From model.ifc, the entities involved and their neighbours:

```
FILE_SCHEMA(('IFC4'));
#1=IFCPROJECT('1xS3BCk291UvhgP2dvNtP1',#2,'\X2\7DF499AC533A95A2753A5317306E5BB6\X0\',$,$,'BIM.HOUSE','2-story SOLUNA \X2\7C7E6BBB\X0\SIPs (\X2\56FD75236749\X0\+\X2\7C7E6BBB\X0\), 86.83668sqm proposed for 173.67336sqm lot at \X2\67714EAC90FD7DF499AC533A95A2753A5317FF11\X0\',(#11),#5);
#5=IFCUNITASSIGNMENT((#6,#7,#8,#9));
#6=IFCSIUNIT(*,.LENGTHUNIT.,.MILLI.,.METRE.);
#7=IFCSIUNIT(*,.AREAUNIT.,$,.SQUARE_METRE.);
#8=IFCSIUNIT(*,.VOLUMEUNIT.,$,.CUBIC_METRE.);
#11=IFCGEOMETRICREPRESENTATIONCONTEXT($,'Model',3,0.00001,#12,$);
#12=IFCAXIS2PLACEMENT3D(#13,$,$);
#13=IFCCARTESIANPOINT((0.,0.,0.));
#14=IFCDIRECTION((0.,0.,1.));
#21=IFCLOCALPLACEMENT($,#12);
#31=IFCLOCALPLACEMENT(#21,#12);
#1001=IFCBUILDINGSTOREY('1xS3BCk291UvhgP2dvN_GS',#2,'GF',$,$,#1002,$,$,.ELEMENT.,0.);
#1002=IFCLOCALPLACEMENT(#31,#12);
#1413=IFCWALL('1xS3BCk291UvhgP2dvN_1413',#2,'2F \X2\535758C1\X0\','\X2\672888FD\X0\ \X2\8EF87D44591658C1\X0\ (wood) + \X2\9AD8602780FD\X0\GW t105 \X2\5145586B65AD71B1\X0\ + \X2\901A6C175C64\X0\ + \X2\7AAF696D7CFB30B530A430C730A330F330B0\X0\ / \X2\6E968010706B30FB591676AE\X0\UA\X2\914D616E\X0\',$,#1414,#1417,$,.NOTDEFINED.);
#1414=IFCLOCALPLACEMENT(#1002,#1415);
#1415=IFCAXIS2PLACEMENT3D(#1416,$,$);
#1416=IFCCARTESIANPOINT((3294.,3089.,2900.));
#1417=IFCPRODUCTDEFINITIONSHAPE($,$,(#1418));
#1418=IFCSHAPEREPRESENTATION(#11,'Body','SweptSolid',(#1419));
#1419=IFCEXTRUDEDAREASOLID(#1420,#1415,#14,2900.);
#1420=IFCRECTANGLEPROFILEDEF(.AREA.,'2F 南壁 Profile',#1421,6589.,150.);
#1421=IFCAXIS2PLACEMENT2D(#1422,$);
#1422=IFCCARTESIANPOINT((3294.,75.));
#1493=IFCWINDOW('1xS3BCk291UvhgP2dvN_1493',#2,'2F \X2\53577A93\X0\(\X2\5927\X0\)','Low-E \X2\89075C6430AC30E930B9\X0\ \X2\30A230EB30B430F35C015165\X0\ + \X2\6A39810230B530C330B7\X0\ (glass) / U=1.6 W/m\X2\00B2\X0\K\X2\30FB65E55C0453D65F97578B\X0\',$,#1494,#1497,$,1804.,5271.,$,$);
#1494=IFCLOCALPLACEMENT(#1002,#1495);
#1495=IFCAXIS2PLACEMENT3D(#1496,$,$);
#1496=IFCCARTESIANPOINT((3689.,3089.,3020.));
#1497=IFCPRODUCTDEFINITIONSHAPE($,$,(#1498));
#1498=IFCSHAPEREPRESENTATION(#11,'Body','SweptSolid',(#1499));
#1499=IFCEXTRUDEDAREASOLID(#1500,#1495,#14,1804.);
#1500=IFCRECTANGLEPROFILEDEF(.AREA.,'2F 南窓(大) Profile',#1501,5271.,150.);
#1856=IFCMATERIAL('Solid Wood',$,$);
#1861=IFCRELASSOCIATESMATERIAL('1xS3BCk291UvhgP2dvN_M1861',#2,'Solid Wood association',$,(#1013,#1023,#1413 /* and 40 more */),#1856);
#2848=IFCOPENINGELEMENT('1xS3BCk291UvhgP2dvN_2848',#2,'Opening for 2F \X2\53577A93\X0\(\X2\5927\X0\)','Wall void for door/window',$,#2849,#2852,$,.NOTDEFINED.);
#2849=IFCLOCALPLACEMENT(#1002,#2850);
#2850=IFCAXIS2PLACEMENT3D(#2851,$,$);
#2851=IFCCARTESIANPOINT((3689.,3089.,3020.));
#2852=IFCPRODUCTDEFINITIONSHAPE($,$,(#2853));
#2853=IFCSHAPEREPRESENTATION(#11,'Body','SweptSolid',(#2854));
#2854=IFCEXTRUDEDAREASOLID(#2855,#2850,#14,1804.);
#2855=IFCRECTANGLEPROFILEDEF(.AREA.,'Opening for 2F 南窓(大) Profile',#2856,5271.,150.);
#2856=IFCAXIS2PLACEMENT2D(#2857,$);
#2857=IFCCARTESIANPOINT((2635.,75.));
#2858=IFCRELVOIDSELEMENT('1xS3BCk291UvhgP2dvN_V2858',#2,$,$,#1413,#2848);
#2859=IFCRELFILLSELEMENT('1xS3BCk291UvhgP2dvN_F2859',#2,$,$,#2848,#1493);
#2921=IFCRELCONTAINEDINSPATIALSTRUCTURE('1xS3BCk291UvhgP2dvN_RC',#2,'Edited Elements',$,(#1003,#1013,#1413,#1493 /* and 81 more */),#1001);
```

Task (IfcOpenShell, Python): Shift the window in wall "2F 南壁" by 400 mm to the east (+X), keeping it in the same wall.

```python
import ifcopenshell
import ifcopenshell.api.geometry
import ifcopenshell.util.placement

model = ifcopenshell.open("model.ifc")

window = model.by_guid("1xS3BCk291UvhgP2dvN_1493")
opening = window.FillsVoids[0].RelatingOpeningElement
wall = opening.VoidsElements[0].RelatingBuildingElement

wall_matrix = ifcopenshell.util.placement.get_local_placement(wall.ObjectPlacement)
shift = wall_matrix[:3, 0] * 400.0
before = ifcopenshell.util.placement.get_local_placement(window.ObjectPlacement)[:3, 3].copy()

# The window is not placed relative to its opening, so move both.
for product in (opening, window):
    matrix = ifcopenshell.util.placement.get_local_placement(product.ObjectPlacement)
    matrix[:3, 3] += shift
    ifcopenshell.api.geometry.edit_object_placement(model, product=product, matrix=matrix, is_si=False)

after = ifcopenshell.util.placement.get_local_placement(window.ObjectPlacement)[:3, 3]
print("window moved by", (after - before).round(3) + 0.0)

model.write("model_edited.ifc")
```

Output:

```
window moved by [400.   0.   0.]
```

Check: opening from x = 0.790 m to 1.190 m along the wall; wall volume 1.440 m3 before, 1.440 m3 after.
